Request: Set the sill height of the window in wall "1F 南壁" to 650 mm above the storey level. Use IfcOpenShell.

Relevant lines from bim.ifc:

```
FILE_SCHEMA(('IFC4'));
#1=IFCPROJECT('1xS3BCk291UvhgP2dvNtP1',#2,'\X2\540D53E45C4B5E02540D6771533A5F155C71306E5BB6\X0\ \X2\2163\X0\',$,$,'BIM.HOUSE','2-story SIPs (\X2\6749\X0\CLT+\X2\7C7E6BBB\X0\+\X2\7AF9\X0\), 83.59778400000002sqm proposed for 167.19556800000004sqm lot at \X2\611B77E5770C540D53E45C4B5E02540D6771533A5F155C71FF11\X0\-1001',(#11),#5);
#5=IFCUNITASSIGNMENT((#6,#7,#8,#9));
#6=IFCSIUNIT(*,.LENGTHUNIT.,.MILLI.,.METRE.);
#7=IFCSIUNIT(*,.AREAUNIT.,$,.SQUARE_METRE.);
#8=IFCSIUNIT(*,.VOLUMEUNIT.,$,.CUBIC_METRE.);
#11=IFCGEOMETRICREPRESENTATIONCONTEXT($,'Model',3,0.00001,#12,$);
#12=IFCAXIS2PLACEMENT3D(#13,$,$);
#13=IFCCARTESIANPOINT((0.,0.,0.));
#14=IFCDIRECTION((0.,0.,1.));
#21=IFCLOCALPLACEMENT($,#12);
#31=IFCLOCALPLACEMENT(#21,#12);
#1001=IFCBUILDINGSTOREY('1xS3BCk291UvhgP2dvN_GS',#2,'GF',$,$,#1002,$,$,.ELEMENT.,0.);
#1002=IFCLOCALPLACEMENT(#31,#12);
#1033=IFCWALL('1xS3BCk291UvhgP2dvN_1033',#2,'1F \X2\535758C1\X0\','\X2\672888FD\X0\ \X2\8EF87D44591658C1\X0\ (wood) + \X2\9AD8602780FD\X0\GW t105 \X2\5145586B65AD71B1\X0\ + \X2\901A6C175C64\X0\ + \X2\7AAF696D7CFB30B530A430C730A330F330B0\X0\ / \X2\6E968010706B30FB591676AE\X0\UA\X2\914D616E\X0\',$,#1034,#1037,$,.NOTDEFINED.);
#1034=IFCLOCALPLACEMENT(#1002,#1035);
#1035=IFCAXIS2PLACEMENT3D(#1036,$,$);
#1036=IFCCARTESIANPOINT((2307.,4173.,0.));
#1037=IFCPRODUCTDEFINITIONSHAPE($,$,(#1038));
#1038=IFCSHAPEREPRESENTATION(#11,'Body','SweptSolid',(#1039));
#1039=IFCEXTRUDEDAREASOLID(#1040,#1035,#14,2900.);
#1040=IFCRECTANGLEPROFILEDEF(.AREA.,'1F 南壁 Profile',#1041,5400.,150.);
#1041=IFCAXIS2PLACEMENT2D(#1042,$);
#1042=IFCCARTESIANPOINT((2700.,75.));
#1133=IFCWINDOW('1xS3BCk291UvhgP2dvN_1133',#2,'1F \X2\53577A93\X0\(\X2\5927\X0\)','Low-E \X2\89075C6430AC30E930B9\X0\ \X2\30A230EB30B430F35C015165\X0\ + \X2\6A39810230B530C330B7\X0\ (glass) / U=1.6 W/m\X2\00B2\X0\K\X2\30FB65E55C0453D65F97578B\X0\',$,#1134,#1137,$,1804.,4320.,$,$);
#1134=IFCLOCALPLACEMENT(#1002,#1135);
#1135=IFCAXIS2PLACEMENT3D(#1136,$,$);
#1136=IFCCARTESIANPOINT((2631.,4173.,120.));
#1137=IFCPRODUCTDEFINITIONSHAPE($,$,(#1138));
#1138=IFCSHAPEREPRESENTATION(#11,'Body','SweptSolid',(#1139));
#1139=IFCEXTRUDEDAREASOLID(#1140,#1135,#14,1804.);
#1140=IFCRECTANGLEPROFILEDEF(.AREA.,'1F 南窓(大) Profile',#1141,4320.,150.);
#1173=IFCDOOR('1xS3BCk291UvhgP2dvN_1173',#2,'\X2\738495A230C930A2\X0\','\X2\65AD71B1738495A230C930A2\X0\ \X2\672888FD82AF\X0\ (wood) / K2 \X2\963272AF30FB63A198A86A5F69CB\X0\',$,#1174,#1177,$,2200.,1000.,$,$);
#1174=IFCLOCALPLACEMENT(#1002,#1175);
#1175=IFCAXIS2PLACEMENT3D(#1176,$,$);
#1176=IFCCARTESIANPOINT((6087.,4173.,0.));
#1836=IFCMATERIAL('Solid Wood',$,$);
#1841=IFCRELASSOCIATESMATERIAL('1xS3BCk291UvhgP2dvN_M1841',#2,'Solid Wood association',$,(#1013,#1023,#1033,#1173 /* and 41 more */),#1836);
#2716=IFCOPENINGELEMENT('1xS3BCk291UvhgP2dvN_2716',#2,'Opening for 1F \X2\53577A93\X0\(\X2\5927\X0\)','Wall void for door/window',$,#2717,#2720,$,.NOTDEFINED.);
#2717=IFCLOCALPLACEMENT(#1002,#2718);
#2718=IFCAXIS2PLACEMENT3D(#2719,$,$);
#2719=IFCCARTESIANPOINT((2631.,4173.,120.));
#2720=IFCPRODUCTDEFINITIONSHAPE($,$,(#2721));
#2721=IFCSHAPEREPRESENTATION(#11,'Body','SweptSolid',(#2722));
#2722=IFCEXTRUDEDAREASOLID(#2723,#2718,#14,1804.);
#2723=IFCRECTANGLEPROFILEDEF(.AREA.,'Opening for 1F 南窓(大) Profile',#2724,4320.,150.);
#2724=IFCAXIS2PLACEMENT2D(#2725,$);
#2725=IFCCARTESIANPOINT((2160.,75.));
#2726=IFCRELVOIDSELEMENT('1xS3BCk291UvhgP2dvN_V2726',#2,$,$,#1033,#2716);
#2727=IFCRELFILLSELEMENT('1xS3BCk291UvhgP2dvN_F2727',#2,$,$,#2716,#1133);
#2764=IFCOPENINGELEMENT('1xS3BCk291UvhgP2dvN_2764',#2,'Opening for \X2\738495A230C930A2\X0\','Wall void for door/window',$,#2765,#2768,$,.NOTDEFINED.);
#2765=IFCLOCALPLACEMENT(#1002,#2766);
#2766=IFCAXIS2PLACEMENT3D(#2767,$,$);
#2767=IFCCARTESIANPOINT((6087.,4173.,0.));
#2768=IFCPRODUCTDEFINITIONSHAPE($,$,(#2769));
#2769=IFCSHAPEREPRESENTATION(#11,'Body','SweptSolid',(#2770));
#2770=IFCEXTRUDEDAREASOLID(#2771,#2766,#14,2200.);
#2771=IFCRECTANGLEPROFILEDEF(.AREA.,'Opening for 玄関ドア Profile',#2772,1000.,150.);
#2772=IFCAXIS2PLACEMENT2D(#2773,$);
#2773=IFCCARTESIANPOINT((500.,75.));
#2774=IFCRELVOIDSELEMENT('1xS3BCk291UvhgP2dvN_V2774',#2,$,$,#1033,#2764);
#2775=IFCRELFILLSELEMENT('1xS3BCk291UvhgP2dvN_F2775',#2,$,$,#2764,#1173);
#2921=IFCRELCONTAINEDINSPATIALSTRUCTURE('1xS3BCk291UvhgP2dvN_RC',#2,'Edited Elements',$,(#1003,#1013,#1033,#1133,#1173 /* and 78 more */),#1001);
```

```python
import numpy as np
import ifcopenshell
import ifcopenshell.api.geometry
import ifcopenshell.geom
import ifcopenshell.util.element
import ifcopenshell.util.placement
import ifcopenshell.util.shape
import ifcopenshell.util.unit

model = ifcopenshell.open("bim.ifc")
unit_scale = ifcopenshell.util.unit.calculate_unit_scale(model)

window = model.by_guid("1xS3BCk291UvhgP2dvN_1133")
opening = window.FillsVoids[0].RelatingOpeningElement
storey = ifcopenshell.util.element.get_container(window, ifc_class="IfcBuildingStorey")
level = ifcopenshell.util.placement.get_local_placement(storey.ObjectPlacement)[2, 3]

# The opening's origin need not be at the sill, so measure its lowest point.
shape = ifcopenshell.geom.create_shape(ifcopenshell.geom.settings(), opening)
bottom = ifcopenshell.util.shape.get_shape_bottom_elevation(shape, shape.geometry) / unit_scale
dz = level + 0.65 / unit_scale - bottom

shift = np.array([0.0, 0.0, dz])
# The window is not placed relative to its opening, so move both.
for product in (opening, window):
    matrix = ifcopenshell.util.placement.get_local_placement(product.ObjectPlacement)
    matrix[:3, 3] += shift
    ifcopenshell.api.geometry.edit_object_placement(model, product=product, matrix=matrix, is_si=False)

print(f"moved by {dz * unit_scale:+.3f} m")

model.write("bim_rev.ifc")
```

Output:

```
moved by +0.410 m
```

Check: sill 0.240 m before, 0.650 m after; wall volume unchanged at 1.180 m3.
